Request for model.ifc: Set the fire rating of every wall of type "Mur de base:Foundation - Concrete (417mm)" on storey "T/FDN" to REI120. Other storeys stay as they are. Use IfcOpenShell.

First a look at what the model holds.

```python
import ifcopenshell
import ifcopenshell.util.element

model = ifcopenshell.open("model.ifc")
print(model.schema)
storey = next(s for s in model.by_type("IfcBuildingStorey") if s.Name == "T/FDN")
walls = [e for e in ifcopenshell.util.element.get_decomposition(storey) if e.is_a("IfcWall")]
seen = {}
for e in walls:
    element_type = ifcopenshell.util.element.get_type(e)
    key = (element_type.Name if element_type != e and element_type else None, ifcopenshell.util.element.get_pset(e, "Pset_WallCommon", "FireRating"))
    seen[key] = seen.get(key, 0) + 1
for (name, value), count in sorted(seen.items(), key=str):
    print(count, "x", name, "|", value)
```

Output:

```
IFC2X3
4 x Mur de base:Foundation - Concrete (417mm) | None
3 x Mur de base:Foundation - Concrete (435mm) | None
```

```python
import ifcopenshell
import ifcopenshell.api.pset
import ifcopenshell.util.element

model = ifcopenshell.open("model.ifc")

storey = next(s for s in model.by_type("IfcBuildingStorey") if s.Name == "T/FDN")
walls = [e for e in ifcopenshell.util.element.get_decomposition(storey) if e.is_a("IfcWall")]

count = 0
for e in walls:
    element_type = ifcopenshell.util.element.get_type(e)
    if element_type in (None, e) or element_type.Name != "Mur de base:Foundation - Concrete (417mm)":
        continue
    # add_pset returns the element's existing set when there is one.
    pset = ifcopenshell.api.pset.add_pset(model, product=e, name="Pset_WallCommon")
    ifcopenshell.api.pset.edit_pset(model, pset=pset, properties={"FireRating": "REI120"})
    count += 1

print(count, "walls updated")

model.write("model_updated.ifc")
```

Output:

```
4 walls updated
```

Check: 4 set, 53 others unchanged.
